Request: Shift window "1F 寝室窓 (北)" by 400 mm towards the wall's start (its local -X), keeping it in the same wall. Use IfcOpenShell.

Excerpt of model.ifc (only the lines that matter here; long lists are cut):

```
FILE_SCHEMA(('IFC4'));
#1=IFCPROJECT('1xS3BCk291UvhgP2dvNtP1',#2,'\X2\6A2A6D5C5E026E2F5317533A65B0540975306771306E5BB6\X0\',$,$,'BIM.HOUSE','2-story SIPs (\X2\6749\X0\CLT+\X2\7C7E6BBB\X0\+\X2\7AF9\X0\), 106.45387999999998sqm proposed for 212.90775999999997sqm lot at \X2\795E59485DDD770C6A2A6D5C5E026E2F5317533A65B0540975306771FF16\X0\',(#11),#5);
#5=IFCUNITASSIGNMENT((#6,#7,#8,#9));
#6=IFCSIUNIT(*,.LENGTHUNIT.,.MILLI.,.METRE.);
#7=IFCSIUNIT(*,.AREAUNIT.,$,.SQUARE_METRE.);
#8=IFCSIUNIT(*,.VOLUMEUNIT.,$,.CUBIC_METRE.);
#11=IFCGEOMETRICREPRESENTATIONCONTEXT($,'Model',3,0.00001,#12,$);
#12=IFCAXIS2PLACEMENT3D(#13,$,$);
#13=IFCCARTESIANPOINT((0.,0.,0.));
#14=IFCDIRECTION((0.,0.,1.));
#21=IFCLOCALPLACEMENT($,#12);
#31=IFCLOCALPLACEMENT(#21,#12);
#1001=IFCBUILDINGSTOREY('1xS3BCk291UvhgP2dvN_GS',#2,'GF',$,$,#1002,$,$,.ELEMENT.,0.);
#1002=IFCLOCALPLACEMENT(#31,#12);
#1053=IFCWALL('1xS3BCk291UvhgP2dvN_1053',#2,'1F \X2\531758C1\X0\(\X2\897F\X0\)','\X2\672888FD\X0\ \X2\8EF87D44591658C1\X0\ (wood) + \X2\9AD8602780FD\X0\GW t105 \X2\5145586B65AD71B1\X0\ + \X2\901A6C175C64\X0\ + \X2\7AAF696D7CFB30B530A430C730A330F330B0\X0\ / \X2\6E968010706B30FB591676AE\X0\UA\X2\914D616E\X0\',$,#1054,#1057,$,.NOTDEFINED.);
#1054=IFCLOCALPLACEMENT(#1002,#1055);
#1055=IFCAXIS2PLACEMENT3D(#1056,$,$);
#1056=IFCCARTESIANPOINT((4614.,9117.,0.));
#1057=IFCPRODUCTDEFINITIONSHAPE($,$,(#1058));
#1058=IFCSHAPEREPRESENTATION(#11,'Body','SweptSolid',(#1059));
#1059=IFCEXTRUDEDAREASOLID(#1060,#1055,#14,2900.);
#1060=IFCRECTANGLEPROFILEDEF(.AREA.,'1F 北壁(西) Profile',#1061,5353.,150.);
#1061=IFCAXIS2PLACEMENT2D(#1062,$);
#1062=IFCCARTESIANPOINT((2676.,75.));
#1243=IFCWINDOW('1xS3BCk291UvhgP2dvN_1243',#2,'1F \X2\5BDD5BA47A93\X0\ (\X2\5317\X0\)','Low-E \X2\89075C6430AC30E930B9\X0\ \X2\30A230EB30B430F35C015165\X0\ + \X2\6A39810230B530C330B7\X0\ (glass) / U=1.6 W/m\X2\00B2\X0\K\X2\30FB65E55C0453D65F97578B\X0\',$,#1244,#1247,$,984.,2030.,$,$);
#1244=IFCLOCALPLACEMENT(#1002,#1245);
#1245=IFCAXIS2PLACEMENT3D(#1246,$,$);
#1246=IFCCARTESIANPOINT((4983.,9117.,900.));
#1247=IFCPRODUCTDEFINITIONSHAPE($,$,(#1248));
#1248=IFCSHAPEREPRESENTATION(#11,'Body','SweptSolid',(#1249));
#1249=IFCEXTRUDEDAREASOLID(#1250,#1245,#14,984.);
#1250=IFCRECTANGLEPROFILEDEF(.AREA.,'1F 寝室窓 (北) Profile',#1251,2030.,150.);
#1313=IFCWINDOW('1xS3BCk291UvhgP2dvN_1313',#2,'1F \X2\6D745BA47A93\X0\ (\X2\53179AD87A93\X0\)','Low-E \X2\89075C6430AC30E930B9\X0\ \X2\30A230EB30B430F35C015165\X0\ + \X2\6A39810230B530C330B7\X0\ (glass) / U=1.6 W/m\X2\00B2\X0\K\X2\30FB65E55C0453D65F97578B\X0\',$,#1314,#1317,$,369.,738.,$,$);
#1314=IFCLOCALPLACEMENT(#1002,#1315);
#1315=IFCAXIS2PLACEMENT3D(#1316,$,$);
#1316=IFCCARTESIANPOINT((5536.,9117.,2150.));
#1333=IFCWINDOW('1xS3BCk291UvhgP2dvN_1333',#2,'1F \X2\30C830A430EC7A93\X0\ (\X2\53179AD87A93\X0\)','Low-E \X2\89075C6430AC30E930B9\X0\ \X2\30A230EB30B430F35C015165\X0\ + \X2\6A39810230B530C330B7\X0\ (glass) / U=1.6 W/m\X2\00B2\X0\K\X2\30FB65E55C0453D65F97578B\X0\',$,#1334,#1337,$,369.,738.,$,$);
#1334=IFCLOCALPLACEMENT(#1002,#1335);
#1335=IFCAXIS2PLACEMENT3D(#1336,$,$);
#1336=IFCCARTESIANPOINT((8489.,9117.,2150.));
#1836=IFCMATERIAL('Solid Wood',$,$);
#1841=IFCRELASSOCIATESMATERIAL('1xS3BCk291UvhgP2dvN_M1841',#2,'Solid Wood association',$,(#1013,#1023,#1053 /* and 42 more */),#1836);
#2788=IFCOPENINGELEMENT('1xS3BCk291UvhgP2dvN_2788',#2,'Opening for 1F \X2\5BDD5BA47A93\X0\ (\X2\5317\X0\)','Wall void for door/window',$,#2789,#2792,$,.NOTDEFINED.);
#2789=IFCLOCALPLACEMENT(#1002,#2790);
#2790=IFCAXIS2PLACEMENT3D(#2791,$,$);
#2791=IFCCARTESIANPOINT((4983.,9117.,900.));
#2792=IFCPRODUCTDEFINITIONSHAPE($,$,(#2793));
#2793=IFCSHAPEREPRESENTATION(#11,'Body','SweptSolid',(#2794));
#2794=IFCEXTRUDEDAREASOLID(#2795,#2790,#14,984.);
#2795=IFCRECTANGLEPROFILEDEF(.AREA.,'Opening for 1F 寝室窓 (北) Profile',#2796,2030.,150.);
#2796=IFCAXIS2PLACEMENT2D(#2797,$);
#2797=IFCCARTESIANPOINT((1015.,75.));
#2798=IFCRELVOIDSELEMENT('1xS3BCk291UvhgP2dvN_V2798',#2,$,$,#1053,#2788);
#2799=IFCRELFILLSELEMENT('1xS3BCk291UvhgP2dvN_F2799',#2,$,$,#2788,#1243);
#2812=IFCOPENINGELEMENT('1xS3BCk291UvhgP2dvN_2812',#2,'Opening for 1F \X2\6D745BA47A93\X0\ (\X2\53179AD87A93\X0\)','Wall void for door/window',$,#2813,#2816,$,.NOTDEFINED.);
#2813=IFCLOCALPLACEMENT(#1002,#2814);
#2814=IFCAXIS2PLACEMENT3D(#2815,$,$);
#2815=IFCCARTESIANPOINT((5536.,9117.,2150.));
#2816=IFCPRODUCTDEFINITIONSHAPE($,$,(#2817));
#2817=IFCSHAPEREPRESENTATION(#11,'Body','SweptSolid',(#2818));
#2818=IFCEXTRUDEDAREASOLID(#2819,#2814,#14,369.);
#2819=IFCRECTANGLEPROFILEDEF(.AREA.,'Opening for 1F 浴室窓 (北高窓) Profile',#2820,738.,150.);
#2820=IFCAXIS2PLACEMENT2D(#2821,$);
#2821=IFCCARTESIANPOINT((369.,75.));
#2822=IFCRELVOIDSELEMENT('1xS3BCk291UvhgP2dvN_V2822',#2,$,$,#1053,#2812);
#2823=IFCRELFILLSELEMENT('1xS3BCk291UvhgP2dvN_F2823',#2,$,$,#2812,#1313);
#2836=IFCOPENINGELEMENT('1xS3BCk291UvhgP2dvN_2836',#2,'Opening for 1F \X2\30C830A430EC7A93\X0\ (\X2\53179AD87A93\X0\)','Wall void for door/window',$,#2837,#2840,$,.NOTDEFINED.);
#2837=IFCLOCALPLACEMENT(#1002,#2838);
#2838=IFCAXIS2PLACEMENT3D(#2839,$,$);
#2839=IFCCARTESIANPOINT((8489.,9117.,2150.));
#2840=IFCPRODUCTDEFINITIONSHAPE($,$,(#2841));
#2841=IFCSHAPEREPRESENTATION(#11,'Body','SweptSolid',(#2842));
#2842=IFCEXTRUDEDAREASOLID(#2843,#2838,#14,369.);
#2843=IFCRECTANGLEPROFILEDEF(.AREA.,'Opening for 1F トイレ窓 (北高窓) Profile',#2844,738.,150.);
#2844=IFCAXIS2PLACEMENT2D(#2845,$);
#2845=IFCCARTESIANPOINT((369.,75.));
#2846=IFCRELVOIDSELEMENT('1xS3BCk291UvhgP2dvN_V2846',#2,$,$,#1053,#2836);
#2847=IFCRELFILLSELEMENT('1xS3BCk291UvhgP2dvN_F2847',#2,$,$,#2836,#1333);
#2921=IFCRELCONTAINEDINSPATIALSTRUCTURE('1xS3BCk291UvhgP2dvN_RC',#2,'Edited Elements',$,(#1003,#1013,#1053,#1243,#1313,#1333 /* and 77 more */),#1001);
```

```python
import ifcopenshell
import ifcopenshell.api.geometry
import ifcopenshell.util.placement

model = ifcopenshell.open("model.ifc")

window = model.by_guid("1xS3BCk291UvhgP2dvN_1243")
opening = window.FillsVoids[0].RelatingOpeningElement
wall = opening.VoidsElements[0].RelatingBuildingElement

wall_matrix = ifcopenshell.util.placement.get_local_placement(wall.ObjectPlacement)
shift = wall_matrix[:3, 0] * -400.0
before = ifcopenshell.util.placement.get_local_placement(window.ObjectPlacement)[:3, 3].copy()

# The window is not placed relative to its opening, so move both.
for product in (opening, window):
    matrix = ifcopenshell.util.placement.get_local_placement(product.ObjectPlacement)
    matrix[:3, 3] += shift
    ifcopenshell.api.geometry.edit_object_placement(model, product=product, matrix=matrix, is_si=False)

after = ifcopenshell.util.placement.get_local_placement(window.ObjectPlacement)[:3, 3]
print("window moved by", (after - before).round(3) + 0.0)

model.write("model-out.ifc")
```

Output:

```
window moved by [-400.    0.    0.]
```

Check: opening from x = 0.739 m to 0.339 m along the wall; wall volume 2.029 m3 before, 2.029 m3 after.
